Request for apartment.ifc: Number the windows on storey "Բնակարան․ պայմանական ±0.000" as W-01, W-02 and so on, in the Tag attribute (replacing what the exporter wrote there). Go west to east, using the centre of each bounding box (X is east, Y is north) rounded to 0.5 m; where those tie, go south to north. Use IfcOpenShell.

First a look at what the model holds.

```python
import ifcopenshell
import ifcopenshell.util.element
import ifcopenshell.util.placement

model = ifcopenshell.open("apartment.ifc")
print(model.schema)
storey = next(s for s in model.by_type("IfcBuildingStorey") if s.Name == "Բնակարան․ պայմանական ±0.000")
windows = [e for e in ifcopenshell.util.element.get_decomposition(storey) if e.is_a("IfcWindow")]
for e in sorted(windows, key=lambda e: e.id()):
    origin = ifcopenshell.util.placement.get_local_placement(e.ObjectPlacement)[:3, 3]
    print(e.id(), e.Tag, e.Name, origin.round(2) + 0.0, sep=" | ")
```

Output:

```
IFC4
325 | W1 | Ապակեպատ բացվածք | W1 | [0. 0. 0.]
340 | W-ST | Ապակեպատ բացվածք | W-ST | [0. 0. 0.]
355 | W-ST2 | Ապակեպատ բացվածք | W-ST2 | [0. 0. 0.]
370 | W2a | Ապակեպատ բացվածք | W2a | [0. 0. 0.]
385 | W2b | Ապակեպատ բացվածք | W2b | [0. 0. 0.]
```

```python
import ifcopenshell
import ifcopenshell.geom
import ifcopenshell.util.element
import ifcopenshell.util.shape

model = ifcopenshell.open("apartment.ifc")
settings = ifcopenshell.geom.settings()
settings.set("use-world-coords", True)


def centre(element):
    shape = ifcopenshell.geom.create_shape(settings, element)
    return ifcopenshell.util.shape.get_bbox_centroid(shape.geometry)


storey = next(s for s in model.by_type("IfcBuildingStorey") if s.Name == "Բնակարան․ պայմանական ±0.000")
windows = [e for e in ifcopenshell.util.element.get_decomposition(storey) if e.is_a("IfcWindow")]

# Insertion points can sit at a corner or the storey origin, so sort by the geometry (in metres).
centres = {e: centre(e) for e in windows}
windows.sort(key=lambda e: (round(centres[e][0] / 0.5), centres[e][1]))

for i, e in enumerate(windows, start=1):
    number = f"W-{i:02d}"
    e.Tag = number
    print(e.id(), number)

model.write("apartment-out.ifc")
```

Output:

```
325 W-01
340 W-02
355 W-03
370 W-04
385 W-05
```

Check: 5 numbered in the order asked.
